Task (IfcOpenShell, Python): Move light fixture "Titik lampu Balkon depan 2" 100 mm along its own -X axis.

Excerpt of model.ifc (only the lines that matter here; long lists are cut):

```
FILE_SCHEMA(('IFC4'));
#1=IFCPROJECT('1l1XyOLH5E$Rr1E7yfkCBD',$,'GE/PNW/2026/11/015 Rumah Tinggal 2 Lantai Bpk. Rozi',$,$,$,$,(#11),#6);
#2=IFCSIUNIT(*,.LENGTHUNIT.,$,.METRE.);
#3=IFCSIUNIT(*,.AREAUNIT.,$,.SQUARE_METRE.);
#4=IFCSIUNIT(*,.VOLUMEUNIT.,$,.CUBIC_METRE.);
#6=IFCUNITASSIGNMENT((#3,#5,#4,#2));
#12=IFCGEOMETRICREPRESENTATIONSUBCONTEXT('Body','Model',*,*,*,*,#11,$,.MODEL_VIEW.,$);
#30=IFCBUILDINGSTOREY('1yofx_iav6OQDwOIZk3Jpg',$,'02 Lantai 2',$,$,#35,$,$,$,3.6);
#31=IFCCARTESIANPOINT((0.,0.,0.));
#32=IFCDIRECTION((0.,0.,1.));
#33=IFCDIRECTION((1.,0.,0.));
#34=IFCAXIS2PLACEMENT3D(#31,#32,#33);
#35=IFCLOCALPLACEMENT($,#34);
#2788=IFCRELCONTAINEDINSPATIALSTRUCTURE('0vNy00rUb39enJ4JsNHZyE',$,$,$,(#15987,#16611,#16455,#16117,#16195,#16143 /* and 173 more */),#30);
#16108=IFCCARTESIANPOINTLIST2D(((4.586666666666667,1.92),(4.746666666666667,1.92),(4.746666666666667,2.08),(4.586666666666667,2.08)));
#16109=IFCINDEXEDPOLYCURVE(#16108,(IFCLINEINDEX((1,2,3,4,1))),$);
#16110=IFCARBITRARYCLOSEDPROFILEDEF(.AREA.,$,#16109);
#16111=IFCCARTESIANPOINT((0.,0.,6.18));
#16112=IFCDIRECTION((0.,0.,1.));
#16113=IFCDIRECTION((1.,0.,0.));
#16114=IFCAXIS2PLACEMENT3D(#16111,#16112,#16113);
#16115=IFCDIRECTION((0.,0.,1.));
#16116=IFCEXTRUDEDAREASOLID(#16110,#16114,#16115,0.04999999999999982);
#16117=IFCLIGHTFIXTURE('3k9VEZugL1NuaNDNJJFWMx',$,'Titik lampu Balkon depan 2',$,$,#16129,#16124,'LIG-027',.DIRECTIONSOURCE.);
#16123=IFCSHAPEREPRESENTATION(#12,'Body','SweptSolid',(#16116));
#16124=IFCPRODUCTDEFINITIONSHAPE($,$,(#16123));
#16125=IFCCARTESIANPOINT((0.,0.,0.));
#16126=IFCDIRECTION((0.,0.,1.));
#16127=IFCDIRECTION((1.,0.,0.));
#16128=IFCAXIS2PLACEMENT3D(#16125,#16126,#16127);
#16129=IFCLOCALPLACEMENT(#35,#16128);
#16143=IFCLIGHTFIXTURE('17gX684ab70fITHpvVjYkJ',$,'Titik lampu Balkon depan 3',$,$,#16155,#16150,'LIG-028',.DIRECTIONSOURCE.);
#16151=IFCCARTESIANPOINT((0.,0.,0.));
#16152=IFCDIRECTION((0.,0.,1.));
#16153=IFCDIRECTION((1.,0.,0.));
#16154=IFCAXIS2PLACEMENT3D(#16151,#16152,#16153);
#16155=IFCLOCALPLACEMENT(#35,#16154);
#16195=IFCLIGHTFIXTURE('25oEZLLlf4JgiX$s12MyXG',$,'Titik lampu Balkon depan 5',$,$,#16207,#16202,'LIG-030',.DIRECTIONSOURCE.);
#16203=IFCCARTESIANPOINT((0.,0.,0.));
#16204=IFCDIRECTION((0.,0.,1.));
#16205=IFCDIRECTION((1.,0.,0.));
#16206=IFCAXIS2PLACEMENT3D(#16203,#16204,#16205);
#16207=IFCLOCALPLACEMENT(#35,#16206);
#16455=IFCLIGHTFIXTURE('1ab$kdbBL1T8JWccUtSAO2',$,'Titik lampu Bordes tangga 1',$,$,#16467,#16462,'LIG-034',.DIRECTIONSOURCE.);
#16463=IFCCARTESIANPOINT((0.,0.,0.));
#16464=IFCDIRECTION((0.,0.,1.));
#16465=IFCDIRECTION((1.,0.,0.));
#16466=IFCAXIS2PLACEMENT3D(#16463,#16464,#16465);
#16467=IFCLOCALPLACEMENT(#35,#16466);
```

```python
import ifcopenshell
import ifcopenshell.api.geometry
import ifcopenshell.util.placement
import ifcopenshell.util.unit

model = ifcopenshell.open("model.ifc")
unit_scale = ifcopenshell.util.unit.calculate_unit_scale(model)

item = model.by_id(16117)
matrix = ifcopenshell.util.placement.get_local_placement(item.ObjectPlacement)
matrix[:3, 3] -= matrix[:3, 0] * 0.1 / unit_scale
ifcopenshell.api.geometry.edit_object_placement(model, product=item, matrix=matrix, is_si=False)

print(ifcopenshell.util.placement.get_local_placement(item.ObjectPlacement).round(3) + 0.0)

model.write("model-out.ifc")
```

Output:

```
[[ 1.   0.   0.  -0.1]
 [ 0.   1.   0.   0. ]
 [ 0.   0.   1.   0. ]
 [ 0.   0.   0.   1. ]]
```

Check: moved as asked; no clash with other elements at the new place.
